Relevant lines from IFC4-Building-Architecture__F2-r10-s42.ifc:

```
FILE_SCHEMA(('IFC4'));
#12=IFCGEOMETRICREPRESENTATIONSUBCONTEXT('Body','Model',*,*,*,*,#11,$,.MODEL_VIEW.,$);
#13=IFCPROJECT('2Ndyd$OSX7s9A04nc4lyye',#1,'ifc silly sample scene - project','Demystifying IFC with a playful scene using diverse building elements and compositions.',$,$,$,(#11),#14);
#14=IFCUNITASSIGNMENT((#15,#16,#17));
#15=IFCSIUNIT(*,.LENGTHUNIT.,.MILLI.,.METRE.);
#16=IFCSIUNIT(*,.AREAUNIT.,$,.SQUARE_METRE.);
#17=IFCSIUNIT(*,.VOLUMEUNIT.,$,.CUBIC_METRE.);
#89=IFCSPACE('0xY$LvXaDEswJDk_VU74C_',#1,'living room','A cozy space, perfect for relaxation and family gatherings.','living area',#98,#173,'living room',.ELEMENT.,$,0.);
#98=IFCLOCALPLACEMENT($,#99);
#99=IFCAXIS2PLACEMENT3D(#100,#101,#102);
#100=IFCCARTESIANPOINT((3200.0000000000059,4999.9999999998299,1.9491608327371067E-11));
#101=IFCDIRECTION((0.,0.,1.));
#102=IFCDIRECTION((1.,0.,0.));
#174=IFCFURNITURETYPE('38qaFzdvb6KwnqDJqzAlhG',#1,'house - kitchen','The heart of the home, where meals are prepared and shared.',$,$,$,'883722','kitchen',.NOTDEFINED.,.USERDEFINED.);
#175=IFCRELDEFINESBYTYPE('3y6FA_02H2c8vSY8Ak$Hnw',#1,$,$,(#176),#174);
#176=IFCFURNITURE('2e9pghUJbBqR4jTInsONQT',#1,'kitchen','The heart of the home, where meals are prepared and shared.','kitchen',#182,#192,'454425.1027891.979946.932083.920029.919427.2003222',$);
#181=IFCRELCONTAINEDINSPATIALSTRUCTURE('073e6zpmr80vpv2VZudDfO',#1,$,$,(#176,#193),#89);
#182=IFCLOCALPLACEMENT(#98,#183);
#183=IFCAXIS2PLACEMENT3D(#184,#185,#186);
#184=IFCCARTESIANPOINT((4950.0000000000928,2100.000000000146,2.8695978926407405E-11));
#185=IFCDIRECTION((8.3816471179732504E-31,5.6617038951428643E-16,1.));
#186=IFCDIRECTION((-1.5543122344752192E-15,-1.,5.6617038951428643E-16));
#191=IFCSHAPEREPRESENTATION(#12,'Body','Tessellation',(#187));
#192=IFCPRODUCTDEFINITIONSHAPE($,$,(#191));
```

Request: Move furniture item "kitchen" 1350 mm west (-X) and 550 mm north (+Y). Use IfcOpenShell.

```python
import ifcopenshell
import ifcopenshell.api.geometry
import ifcopenshell.util.placement
import ifcopenshell.util.unit

model = ifcopenshell.open("IFC4-Building-Architecture__F2-r10-s42.ifc")
unit_scale = ifcopenshell.util.unit.calculate_unit_scale(model)

item = model.by_guid("2e9pghUJbBqR4jTInsONQT")
matrix = ifcopenshell.util.placement.get_local_placement(item.ObjectPlacement)
matrix[0, 3] -= 1.35 / unit_scale
matrix[1, 3] += 0.55 / unit_scale
ifcopenshell.api.geometry.edit_object_placement(model, product=item, matrix=matrix, is_si=False)

print(ifcopenshell.util.placement.get_local_placement(item.ObjectPlacement).round(3) + 0.0)

model.write("IFC4-Building-Architecture__F2-r10-s42_rev.ifc")
```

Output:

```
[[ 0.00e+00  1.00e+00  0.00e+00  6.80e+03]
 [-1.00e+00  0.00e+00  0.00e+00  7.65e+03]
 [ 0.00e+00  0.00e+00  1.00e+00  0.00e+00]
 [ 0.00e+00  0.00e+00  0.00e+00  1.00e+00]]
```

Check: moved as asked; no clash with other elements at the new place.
